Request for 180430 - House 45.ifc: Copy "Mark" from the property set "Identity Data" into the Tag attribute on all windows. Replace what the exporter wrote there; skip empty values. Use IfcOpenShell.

First a look at what the model holds.

```python
import ifcopenshell
import ifcopenshell.util.element

model = ifcopenshell.open("180430 - House 45.ifc")
print(model.schema)
windows = model.by_type("IfcWindow")
print(len(windows), "windows")
for e in windows[:8]:
    source = ifcopenshell.util.element.get_pset(e, "Identity Data", "Mark")
    target = e.Tag
    print(e.id(), repr(source), repr(target), sep=" | ")
```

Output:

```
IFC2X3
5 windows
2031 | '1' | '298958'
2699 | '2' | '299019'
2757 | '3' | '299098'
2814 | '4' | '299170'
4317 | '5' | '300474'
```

```python
import ifcopenshell
import ifcopenshell.util.element

model = ifcopenshell.open("180430 - House 45.ifc")

count = 0
for e in model.by_type("IfcWindow"):
    value = ifcopenshell.util.element.get_pset(e, "Identity Data", "Mark")
    current = e.Tag
    if not value or not value.strip() or current == value:
        continue
    e.Tag = value
    count += 1

print(count, "windows updated")

model.write("180430 - House 45_edited.ifc")
```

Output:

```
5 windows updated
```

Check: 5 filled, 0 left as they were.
